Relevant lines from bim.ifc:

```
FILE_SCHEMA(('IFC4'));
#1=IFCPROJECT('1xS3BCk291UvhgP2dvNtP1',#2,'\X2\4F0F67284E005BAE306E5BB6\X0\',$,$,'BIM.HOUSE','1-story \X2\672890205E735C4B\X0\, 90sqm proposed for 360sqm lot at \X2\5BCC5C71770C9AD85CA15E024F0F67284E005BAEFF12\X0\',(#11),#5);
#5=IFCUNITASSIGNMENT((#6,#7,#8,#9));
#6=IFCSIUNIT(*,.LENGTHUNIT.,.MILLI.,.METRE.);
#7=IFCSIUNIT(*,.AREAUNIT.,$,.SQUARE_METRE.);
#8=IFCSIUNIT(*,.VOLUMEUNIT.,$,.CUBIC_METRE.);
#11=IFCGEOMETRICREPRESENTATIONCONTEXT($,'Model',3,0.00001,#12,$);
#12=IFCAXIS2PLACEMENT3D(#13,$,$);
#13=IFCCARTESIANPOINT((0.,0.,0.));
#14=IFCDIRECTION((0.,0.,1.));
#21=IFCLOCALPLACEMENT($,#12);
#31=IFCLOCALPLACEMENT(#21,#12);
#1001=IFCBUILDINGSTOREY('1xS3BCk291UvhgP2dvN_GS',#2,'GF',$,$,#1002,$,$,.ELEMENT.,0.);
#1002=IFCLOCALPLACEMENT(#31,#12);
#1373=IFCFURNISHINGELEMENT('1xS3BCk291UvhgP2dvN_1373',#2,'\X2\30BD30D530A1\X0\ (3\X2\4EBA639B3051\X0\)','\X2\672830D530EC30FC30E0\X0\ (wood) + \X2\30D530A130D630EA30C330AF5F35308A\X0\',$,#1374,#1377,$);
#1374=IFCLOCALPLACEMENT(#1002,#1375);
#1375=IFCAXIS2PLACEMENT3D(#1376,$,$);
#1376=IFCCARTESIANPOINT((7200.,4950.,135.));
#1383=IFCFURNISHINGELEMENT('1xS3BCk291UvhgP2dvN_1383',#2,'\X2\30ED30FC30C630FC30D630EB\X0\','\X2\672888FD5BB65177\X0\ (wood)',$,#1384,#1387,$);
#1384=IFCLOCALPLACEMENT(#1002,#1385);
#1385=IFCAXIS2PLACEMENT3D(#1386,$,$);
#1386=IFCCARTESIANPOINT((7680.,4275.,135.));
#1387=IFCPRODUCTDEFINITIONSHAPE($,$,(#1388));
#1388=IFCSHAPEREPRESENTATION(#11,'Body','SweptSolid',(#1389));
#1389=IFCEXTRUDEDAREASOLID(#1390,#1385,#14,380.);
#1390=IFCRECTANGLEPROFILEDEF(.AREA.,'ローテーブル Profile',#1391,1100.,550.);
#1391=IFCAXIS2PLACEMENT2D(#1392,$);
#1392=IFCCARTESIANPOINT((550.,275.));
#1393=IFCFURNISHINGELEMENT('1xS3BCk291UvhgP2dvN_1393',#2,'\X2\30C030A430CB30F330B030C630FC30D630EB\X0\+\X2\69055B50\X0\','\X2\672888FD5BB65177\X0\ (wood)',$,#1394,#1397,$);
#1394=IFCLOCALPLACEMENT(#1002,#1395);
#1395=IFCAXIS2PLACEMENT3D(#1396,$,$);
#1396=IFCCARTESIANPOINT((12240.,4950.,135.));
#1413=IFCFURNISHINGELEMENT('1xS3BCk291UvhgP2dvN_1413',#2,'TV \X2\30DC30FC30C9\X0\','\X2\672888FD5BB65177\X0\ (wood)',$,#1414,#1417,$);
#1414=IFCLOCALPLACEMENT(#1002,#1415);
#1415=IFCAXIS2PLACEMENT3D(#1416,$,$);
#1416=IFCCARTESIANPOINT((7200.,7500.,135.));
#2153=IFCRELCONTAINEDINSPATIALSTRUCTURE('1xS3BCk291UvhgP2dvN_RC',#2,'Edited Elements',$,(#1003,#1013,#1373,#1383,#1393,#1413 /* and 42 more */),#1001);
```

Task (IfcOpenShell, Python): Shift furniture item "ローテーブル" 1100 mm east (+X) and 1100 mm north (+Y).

```python
import ifcopenshell
import ifcopenshell.api.geometry
import ifcopenshell.util.placement
import ifcopenshell.util.unit

model = ifcopenshell.open("bim.ifc")
unit_scale = ifcopenshell.util.unit.calculate_unit_scale(model)

item = model.by_guid("1xS3BCk291UvhgP2dvN_1383")
matrix = ifcopenshell.util.placement.get_local_placement(item.ObjectPlacement)
matrix[0, 3] += 1.1 / unit_scale
matrix[1, 3] += 1.1 / unit_scale
ifcopenshell.api.geometry.edit_object_placement(model, product=item, matrix=matrix, is_si=False)

print(ifcopenshell.util.placement.get_local_placement(item.ObjectPlacement).round(3) + 0.0)

model.write("bim_edited.ifc")
```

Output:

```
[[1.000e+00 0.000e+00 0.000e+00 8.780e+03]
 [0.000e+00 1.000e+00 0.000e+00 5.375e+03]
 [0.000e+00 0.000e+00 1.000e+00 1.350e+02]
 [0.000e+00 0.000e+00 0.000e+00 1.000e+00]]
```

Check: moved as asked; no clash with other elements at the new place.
